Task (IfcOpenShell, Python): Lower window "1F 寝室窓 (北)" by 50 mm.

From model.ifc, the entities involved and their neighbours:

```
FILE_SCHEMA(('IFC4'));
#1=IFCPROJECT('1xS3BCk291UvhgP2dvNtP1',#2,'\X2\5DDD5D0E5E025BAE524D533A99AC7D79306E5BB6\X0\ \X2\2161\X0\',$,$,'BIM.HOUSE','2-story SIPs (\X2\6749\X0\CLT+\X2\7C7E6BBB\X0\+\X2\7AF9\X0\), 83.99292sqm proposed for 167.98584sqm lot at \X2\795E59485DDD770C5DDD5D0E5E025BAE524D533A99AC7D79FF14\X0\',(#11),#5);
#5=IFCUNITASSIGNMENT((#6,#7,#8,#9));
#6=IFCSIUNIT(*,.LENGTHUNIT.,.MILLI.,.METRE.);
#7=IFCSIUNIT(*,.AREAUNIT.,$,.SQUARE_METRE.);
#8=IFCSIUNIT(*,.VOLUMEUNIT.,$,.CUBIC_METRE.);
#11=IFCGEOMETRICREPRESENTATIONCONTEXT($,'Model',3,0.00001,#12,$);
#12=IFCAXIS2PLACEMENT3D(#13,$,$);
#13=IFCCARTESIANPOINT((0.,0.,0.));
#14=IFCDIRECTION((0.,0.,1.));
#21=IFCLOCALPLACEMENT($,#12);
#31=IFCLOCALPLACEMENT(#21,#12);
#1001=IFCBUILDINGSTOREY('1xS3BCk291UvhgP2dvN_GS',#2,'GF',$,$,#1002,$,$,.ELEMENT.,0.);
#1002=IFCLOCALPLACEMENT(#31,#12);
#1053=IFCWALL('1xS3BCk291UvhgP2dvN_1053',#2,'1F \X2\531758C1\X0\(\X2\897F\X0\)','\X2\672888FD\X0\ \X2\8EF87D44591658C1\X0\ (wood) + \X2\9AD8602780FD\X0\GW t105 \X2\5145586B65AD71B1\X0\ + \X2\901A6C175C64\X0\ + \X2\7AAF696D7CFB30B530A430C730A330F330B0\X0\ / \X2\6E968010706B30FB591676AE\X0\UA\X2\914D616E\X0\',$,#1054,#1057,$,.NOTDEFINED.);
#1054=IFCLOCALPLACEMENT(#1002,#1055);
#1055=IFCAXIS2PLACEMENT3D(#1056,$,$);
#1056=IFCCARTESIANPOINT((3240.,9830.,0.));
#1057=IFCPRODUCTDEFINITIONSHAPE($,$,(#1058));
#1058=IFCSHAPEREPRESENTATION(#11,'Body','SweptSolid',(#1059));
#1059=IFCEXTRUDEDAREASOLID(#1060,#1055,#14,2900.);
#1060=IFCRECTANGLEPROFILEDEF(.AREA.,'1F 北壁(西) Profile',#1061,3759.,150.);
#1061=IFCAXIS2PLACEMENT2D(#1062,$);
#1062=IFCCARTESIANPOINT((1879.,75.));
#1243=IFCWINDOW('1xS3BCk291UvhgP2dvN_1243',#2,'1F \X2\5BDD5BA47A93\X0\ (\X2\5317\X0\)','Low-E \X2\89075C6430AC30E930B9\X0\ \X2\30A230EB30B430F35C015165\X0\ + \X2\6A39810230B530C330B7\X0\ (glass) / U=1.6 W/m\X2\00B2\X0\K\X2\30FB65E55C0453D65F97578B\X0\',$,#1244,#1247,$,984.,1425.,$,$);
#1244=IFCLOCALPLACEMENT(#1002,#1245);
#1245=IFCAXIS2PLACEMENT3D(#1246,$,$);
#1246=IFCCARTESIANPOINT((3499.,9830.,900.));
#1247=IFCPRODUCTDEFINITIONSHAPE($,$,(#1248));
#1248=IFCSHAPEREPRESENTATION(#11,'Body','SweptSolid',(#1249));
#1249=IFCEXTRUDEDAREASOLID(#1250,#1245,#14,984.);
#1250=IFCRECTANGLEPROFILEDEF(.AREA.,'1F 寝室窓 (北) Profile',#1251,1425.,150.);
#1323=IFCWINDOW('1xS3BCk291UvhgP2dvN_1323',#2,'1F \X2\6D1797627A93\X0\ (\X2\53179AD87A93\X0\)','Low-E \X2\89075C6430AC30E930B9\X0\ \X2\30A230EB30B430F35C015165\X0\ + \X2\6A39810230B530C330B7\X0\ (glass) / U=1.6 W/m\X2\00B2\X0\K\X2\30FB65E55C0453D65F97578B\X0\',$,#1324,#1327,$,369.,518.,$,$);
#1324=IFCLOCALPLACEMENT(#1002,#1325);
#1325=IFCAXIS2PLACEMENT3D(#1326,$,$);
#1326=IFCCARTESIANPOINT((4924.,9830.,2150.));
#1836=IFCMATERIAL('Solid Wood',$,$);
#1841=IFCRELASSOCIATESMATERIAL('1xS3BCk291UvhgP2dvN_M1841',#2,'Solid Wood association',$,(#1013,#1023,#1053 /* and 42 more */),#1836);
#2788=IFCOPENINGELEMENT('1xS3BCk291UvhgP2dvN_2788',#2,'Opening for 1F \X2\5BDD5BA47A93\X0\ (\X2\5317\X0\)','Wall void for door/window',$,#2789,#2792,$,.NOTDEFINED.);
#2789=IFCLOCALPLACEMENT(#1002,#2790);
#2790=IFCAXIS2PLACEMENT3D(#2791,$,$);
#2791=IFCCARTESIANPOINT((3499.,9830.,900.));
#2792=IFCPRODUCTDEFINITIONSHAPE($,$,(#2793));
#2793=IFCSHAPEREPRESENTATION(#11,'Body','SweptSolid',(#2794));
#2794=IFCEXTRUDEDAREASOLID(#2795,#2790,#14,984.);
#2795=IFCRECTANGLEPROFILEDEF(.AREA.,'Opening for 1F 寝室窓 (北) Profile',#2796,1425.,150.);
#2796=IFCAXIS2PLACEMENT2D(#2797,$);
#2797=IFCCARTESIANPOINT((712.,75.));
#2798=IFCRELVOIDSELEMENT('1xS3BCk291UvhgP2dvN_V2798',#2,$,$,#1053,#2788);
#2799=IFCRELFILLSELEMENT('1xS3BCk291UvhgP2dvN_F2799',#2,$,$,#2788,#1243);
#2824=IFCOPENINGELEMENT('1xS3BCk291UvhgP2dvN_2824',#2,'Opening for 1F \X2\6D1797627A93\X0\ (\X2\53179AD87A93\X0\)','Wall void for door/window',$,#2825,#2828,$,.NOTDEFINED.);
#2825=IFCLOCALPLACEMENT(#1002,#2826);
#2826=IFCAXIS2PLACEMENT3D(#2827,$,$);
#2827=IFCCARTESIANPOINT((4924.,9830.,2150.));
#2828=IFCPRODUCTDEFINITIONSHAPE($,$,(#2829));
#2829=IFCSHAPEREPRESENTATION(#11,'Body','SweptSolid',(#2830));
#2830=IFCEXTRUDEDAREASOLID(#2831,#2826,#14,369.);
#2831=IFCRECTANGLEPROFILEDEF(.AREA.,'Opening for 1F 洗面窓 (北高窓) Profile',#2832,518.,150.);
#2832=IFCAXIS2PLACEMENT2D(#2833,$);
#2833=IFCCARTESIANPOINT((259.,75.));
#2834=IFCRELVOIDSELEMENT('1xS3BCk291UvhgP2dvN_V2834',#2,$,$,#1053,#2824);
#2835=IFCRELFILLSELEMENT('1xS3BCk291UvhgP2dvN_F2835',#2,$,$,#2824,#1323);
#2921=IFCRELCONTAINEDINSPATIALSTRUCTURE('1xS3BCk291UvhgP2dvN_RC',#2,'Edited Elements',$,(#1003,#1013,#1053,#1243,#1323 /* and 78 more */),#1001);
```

```python
import numpy as np
import ifcopenshell
import ifcopenshell.api.geometry
import ifcopenshell.util.placement
import ifcopenshell.util.unit

model = ifcopenshell.open("model.ifc")
unit_scale = ifcopenshell.util.unit.calculate_unit_scale(model)

window = model.by_guid("1xS3BCk291UvhgP2dvN_1243")
opening = window.FillsVoids[0].RelatingOpeningElement
dz = -0.05 / unit_scale

shift = np.array([0.0, 0.0, dz])
# The window is not placed relative to its opening, so move both.
for product in (opening, window):
    matrix = ifcopenshell.util.placement.get_local_placement(product.ObjectPlacement)
    matrix[:3, 3] += shift
    ifcopenshell.api.geometry.edit_object_placement(model, product=product, matrix=matrix, is_si=False)

print(f"moved by {dz * unit_scale:+.3f} m")

model.write("model_updated.ifc")
```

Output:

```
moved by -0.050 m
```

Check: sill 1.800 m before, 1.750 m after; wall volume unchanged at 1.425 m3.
